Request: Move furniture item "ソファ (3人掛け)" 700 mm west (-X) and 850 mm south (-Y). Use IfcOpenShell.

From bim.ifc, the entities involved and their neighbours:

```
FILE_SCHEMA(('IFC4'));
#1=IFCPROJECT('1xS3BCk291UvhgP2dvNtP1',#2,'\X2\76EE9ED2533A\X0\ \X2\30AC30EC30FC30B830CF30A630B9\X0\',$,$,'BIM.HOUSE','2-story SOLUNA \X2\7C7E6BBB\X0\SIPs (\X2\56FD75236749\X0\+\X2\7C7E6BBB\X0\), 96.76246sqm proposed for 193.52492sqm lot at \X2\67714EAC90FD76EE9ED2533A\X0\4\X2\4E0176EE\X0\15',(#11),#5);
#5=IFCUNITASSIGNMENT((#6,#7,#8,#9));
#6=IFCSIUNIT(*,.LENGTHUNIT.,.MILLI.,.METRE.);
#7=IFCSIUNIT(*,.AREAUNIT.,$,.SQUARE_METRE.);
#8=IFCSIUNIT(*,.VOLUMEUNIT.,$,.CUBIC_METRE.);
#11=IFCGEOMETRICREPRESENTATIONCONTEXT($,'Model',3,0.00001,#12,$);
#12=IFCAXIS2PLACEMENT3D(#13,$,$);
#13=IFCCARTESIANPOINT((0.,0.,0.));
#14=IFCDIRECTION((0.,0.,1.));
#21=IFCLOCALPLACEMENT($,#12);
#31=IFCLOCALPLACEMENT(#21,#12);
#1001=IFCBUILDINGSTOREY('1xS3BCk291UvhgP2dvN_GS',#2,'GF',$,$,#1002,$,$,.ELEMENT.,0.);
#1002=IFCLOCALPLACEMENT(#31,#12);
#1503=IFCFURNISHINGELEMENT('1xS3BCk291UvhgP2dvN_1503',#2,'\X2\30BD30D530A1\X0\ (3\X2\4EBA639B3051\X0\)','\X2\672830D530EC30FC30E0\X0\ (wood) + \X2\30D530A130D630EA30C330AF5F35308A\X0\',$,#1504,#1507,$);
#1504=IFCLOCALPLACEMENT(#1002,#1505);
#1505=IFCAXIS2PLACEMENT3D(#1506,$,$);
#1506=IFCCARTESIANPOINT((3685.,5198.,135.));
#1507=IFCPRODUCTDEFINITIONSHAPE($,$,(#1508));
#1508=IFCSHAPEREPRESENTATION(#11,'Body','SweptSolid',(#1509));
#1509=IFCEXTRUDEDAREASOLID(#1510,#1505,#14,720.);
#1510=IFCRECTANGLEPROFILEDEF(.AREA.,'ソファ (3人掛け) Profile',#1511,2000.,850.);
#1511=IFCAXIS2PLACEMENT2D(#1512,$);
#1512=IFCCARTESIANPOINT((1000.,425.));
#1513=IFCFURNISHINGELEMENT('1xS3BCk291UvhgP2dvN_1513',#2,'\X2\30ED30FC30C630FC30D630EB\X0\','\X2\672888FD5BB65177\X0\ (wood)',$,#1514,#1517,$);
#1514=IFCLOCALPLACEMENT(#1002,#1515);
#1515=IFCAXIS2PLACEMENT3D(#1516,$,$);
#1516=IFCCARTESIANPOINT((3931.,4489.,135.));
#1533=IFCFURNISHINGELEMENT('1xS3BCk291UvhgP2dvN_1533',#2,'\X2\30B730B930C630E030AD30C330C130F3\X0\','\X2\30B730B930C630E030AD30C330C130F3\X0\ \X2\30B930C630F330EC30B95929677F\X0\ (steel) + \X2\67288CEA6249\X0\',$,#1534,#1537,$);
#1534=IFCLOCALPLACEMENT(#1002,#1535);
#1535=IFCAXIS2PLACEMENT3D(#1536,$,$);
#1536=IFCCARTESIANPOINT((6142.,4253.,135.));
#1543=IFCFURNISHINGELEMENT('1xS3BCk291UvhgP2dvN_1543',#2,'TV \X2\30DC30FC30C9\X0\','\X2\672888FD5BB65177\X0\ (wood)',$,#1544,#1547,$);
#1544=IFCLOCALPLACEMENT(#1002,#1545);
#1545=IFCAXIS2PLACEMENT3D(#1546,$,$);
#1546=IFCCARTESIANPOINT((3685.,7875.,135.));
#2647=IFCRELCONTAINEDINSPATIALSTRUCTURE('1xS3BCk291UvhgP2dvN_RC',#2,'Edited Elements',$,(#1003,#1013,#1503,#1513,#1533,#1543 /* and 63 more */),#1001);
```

```python
import ifcopenshell
import ifcopenshell.api.geometry
import ifcopenshell.util.placement
import ifcopenshell.util.unit

model = ifcopenshell.open("bim.ifc")
unit_scale = ifcopenshell.util.unit.calculate_unit_scale(model)

item = model.by_id(1503)
matrix = ifcopenshell.util.placement.get_local_placement(item.ObjectPlacement)
matrix[0, 3] -= 0.7 / unit_scale
matrix[1, 3] -= 0.85 / unit_scale
ifcopenshell.api.geometry.edit_object_placement(model, product=item, matrix=matrix, is_si=False)

print(ifcopenshell.util.placement.get_local_placement(item.ObjectPlacement).round(3) + 0.0)

model.write("bim_updated.ifc")
```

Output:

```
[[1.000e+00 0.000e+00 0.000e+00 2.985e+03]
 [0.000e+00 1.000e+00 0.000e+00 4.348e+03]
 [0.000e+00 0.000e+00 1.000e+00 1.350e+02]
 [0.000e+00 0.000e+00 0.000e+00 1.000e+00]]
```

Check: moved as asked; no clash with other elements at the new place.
